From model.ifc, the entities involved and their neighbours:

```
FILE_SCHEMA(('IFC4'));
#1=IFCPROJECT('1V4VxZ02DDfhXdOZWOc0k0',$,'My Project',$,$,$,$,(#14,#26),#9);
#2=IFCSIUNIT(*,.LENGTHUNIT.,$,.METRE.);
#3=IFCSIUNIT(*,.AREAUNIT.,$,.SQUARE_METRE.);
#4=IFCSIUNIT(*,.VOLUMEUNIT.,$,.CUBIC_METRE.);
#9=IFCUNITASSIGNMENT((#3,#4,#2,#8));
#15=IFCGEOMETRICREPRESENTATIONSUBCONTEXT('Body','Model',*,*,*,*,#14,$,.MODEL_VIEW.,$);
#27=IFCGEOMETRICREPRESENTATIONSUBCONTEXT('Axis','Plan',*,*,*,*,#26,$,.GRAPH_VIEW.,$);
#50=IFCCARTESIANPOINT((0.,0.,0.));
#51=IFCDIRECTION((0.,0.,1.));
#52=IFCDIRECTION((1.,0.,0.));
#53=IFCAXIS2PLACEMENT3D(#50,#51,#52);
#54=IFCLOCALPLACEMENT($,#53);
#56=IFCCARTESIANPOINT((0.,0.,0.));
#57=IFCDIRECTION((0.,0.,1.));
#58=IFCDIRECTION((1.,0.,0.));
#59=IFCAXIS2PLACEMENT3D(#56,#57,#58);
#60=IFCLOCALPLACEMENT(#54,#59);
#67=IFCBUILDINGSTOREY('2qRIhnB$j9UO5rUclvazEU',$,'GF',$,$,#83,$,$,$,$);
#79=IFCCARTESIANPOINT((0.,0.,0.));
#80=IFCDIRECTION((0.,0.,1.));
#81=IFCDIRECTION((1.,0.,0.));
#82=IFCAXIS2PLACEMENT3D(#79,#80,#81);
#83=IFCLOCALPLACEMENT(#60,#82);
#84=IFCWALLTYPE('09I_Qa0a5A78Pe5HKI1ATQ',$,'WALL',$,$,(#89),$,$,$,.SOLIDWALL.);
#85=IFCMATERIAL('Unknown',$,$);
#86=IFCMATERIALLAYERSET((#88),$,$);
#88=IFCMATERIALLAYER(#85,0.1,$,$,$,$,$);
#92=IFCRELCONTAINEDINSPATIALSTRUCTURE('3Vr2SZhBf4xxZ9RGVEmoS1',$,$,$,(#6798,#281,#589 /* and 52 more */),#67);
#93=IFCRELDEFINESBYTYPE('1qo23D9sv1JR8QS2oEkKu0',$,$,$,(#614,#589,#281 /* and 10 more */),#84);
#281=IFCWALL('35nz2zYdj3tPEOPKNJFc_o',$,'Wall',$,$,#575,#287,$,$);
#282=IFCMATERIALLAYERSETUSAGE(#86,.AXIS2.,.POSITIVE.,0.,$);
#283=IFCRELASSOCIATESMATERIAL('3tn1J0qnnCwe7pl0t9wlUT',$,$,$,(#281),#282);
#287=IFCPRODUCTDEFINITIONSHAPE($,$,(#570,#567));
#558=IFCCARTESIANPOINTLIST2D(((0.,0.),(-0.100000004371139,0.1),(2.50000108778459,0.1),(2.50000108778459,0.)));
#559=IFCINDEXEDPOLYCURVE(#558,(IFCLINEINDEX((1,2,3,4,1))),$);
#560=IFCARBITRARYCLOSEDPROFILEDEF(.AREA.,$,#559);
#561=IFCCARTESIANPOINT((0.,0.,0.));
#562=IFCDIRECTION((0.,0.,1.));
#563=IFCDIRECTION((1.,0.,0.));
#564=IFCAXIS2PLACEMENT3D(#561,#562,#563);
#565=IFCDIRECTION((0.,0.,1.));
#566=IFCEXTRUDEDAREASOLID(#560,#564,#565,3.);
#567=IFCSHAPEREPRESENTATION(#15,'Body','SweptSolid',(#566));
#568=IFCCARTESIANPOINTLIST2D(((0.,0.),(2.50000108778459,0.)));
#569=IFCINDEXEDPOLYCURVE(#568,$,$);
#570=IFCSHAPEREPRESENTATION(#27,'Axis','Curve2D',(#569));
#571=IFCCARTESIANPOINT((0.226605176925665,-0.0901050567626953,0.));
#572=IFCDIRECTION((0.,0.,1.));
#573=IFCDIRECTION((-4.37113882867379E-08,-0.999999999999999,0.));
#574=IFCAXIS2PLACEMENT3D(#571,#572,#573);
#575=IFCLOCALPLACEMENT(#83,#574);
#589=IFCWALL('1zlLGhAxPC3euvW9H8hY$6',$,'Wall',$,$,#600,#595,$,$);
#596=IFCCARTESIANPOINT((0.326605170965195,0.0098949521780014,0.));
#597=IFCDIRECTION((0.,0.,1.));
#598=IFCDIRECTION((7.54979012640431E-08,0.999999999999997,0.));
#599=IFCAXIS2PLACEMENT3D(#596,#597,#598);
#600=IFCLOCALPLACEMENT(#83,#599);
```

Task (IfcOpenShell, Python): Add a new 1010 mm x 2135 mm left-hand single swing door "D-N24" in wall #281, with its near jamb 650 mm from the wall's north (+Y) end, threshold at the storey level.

```python
import numpy as np
import ifcopenshell
import ifcopenshell.api.feature
import ifcopenshell.api.geometry
import ifcopenshell.api.root
import ifcopenshell.api.spatial
import ifcopenshell.geom
import ifcopenshell.util.element
import ifcopenshell.util.placement
import ifcopenshell.util.representation
import ifcopenshell.util.shape
import ifcopenshell.util.unit

model = ifcopenshell.open("model.ifc")
unit_scale = ifcopenshell.util.unit.calculate_unit_scale(model)
settings = ifcopenshell.geom.settings()


def volume(element):
    """Net volume in cubic metres, openings subtracted."""
    shape = ifcopenshell.geom.create_shape(settings, element)
    return ifcopenshell.util.shape.get_volume(shape.geometry)


wall = model.by_guid("35nz2zYdj3tPEOPKNJFc_o")
storey = ifcopenshell.util.element.get_container(wall, ifc_class="IfcBuildingStorey")
context = ifcopenshell.util.representation.get_context(model, "Model", "Body", "MODEL_VIEW")
before = volume(wall)

width, height, from_end, sill = 1.01, 2.135, 0.65, 0.0  # metres

# The wall runs along its own X axis, and the end named is its -X end.
wall_shape = ifcopenshell.geom.create_shape(settings, wall)
x, y, z = ifcopenshell.util.shape.get_vertices(wall_shape.geometry).T
start = x.min() + from_end
face, thickness = float(y.min()), float(y.max() - y.min())
wall_matrix = ifcopenshell.util.placement.get_local_placement(wall.ObjectPlacement)
level = ifcopenshell.util.placement.get_local_placement(storey.ObjectPlacement)[2, 3]


def in_wall(x, y):
    """Placement at x, y metres in the wall's axes, at sill height."""
    matrix = wall_matrix.copy()
    matrix[:, 3] = wall_matrix @ np.array([x / unit_scale, y / unit_scale, 0.0, 1.0])
    matrix[2, 3] = level + sill / unit_scale
    return matrix


# Opening: a box that overshoots both wall faces by 50 mm.
opening = ifcopenshell.api.root.create_entity(model, ifc_class="IfcOpeningElement", predefined_type="OPENING")
box = ifcopenshell.api.geometry.add_wall_representation(
    model, context=context, length=width, height=height, thickness=thickness + 0.1
)
ifcopenshell.api.geometry.assign_representation(model, product=opening, representation=box)
ifcopenshell.api.geometry.edit_object_placement(model, product=opening, matrix=in_wall(start, face - 0.05), is_si=False)
ifcopenshell.api.feature.add_feature(model, feature=opening, element=wall)

door = ifcopenshell.api.root.create_entity(model, ifc_class="IfcDoor", name="D-N24", predefined_type="DOOR")
door.OverallWidth, door.OverallHeight = width / unit_scale, height / unit_scale
door.OperationType = "SINGLE_SWING_LEFT"
body = ifcopenshell.api.geometry.add_door_representation(
    model,
    context=context,
    overall_width=door.OverallWidth,
    overall_height=door.OverallHeight,
    operation_type="SINGLE_SWING_LEFT",
    lining_properties={"LiningDepth": thickness / unit_scale, "ThresholdDepth": thickness / unit_scale},
)
ifcopenshell.api.geometry.assign_representation(model, product=door, representation=body)
ifcopenshell.api.spatial.assign_container(model, products=[door], relating_structure=storey)
ifcopenshell.api.feature.add_filling(model, opening=opening, element=door)

# The lining spans the wall, so the door starts at the wall face.
ifcopenshell.api.geometry.edit_object_placement(model, product=door, matrix=in_wall(start, face), is_si=False)

after = volume(wall)

print(f"wall volume {before:.3f} -> {after:.3f} m3")

model.write("model_updated.ifc")
```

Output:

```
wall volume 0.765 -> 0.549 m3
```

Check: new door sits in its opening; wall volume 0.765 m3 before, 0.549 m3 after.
